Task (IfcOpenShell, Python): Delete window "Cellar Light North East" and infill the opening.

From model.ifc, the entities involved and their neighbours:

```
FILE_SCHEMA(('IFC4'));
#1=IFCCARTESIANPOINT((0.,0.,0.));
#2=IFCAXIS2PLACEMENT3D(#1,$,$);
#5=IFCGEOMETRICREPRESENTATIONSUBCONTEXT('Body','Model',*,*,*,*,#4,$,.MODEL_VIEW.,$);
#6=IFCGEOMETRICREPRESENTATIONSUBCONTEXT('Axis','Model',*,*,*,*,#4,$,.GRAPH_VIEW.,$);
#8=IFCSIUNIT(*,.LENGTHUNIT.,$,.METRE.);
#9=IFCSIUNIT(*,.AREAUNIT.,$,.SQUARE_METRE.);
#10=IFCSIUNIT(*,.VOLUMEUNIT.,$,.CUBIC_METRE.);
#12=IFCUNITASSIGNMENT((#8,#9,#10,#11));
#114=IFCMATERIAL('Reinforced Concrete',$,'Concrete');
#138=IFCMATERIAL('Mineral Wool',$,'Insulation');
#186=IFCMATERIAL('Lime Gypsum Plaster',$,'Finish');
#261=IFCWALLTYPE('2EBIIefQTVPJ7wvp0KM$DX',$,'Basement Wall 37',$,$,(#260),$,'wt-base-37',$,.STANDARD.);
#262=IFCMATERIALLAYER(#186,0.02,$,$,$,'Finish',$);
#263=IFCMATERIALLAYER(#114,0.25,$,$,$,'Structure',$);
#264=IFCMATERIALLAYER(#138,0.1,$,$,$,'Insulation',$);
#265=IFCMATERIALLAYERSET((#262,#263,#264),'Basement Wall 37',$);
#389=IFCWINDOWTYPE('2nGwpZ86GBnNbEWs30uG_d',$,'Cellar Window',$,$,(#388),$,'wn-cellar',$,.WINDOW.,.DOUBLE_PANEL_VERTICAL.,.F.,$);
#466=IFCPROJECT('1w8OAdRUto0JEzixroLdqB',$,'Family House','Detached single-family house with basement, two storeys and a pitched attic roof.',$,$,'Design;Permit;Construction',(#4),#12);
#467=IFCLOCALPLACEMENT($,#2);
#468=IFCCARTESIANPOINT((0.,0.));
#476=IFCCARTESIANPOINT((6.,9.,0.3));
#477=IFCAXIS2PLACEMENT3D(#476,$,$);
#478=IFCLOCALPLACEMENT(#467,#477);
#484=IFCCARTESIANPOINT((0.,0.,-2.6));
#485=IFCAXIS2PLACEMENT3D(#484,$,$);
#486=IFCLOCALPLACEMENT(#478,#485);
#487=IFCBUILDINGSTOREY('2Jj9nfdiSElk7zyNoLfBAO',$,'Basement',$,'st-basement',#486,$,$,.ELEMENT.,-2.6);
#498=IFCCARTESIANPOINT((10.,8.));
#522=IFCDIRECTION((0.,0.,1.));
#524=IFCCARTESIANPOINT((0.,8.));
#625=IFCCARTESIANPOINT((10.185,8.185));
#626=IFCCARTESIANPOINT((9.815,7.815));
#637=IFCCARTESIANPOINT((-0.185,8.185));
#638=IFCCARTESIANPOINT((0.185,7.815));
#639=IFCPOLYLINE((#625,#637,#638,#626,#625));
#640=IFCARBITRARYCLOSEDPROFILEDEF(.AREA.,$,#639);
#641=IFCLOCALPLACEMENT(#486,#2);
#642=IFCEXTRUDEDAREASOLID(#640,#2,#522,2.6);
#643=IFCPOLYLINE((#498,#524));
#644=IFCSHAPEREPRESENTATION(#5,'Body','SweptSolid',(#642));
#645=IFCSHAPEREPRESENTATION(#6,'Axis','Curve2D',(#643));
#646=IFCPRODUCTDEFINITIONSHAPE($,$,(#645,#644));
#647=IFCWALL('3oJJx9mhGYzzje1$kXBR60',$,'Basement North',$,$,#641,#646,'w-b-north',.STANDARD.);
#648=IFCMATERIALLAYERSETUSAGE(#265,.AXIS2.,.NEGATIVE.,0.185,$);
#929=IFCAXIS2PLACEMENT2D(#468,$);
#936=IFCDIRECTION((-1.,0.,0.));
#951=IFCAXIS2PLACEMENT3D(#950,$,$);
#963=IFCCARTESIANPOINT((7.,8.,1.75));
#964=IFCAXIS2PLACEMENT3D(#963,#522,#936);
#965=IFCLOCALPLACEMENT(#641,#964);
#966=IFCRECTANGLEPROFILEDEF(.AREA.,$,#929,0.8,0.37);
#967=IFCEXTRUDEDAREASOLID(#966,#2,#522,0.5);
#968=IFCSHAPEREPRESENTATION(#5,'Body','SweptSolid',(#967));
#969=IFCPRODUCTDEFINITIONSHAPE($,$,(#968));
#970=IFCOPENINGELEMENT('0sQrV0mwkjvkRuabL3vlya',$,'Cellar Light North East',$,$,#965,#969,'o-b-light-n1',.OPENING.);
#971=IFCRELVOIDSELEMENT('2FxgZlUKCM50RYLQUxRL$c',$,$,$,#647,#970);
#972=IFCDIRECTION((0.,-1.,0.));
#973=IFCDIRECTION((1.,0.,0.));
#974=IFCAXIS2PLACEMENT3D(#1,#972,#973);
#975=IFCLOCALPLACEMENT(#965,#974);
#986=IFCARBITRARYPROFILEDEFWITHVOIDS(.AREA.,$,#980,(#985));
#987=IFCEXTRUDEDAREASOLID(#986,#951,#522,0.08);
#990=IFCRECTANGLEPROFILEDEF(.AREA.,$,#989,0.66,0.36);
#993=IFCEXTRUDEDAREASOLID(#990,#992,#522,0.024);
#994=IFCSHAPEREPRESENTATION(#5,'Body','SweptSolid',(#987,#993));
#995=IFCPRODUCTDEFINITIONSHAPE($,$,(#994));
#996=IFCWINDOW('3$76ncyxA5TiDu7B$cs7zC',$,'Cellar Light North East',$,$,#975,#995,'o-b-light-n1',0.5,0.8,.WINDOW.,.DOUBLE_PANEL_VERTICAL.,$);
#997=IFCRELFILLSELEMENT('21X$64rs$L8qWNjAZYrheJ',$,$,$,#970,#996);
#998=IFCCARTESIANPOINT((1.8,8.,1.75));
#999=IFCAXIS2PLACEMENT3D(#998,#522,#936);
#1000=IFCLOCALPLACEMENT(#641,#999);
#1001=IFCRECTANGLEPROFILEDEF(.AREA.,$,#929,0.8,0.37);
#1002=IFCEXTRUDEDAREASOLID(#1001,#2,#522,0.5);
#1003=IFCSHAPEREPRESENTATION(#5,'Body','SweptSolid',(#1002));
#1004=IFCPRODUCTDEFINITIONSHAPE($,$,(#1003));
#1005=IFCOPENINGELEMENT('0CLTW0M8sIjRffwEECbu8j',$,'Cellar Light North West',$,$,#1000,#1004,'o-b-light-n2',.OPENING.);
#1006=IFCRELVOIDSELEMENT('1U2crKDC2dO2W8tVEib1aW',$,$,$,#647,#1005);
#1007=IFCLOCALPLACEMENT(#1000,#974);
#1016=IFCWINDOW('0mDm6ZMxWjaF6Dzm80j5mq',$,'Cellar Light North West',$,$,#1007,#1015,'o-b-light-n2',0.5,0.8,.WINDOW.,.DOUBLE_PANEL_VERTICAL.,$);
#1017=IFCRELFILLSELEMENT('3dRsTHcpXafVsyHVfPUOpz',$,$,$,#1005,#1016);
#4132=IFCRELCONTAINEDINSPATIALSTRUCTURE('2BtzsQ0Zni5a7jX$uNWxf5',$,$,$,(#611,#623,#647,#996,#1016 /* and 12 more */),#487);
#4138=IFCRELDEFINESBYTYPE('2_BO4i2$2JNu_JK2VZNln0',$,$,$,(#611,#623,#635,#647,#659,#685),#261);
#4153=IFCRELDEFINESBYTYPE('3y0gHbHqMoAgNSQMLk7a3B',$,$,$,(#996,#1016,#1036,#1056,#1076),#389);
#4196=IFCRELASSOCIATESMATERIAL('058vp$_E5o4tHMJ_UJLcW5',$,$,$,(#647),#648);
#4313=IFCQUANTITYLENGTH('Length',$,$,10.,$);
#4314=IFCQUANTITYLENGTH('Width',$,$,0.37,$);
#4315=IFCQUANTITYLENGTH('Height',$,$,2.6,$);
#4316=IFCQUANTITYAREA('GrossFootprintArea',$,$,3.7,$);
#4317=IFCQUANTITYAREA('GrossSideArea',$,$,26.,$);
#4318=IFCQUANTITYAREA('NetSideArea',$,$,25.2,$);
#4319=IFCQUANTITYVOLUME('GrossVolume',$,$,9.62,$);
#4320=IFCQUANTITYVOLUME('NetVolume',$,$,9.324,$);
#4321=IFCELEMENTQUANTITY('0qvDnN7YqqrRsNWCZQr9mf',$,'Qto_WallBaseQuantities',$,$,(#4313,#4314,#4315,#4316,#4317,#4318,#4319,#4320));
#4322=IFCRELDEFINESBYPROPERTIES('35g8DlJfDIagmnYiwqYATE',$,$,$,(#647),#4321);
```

```python
import ifcopenshell
import ifcopenshell.api.feature
import ifcopenshell.api.pset
import ifcopenshell.api.root
import ifcopenshell.geom
import ifcopenshell.util.element
import ifcopenshell.util.shape
import ifcopenshell.util.unit

model = ifcopenshell.open("model.ifc")
area_scale = ifcopenshell.util.unit.calculate_unit_scale(model, "AREAUNIT")
volume_scale = ifcopenshell.util.unit.calculate_unit_scale(model, "VOLUMEUNIT")
settings = ifcopenshell.geom.settings()


def volume(element):
    """Net volume in cubic metres, openings subtracted."""
    shape = ifcopenshell.geom.create_shape(settings, element)
    return ifcopenshell.util.shape.get_volume(shape.geometry)


window = model.by_id(996)
opening = window.FillsVoids[0].RelatingOpeningElement
wall = opening.VoidsElements[0].RelatingBuildingElement
before = volume(wall)

ifcopenshell.api.root.remove_product(model, product=window)
ifcopenshell.api.feature.remove_feature(model, feature=opening)

after = volume(wall)
thickness = 0.37  # wall thickness in metres

# Update the wall's stored quantities.
qto = model.by_id(ifcopenshell.util.element.get_pset(wall, "Qto_WallBaseQuantities", should_inherit=False)["id"])
ifcopenshell.api.pset.edit_qto(model, qto=qto, properties={
    "NetSideArea": after / thickness / area_scale,
    "NetVolume": after / volume_scale,
})

print(f"wall volume {before:.3f} -> {after:.3f} m3")

model.write("model-out.ifc")
```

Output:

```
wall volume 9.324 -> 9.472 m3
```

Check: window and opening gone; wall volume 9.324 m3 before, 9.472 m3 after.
